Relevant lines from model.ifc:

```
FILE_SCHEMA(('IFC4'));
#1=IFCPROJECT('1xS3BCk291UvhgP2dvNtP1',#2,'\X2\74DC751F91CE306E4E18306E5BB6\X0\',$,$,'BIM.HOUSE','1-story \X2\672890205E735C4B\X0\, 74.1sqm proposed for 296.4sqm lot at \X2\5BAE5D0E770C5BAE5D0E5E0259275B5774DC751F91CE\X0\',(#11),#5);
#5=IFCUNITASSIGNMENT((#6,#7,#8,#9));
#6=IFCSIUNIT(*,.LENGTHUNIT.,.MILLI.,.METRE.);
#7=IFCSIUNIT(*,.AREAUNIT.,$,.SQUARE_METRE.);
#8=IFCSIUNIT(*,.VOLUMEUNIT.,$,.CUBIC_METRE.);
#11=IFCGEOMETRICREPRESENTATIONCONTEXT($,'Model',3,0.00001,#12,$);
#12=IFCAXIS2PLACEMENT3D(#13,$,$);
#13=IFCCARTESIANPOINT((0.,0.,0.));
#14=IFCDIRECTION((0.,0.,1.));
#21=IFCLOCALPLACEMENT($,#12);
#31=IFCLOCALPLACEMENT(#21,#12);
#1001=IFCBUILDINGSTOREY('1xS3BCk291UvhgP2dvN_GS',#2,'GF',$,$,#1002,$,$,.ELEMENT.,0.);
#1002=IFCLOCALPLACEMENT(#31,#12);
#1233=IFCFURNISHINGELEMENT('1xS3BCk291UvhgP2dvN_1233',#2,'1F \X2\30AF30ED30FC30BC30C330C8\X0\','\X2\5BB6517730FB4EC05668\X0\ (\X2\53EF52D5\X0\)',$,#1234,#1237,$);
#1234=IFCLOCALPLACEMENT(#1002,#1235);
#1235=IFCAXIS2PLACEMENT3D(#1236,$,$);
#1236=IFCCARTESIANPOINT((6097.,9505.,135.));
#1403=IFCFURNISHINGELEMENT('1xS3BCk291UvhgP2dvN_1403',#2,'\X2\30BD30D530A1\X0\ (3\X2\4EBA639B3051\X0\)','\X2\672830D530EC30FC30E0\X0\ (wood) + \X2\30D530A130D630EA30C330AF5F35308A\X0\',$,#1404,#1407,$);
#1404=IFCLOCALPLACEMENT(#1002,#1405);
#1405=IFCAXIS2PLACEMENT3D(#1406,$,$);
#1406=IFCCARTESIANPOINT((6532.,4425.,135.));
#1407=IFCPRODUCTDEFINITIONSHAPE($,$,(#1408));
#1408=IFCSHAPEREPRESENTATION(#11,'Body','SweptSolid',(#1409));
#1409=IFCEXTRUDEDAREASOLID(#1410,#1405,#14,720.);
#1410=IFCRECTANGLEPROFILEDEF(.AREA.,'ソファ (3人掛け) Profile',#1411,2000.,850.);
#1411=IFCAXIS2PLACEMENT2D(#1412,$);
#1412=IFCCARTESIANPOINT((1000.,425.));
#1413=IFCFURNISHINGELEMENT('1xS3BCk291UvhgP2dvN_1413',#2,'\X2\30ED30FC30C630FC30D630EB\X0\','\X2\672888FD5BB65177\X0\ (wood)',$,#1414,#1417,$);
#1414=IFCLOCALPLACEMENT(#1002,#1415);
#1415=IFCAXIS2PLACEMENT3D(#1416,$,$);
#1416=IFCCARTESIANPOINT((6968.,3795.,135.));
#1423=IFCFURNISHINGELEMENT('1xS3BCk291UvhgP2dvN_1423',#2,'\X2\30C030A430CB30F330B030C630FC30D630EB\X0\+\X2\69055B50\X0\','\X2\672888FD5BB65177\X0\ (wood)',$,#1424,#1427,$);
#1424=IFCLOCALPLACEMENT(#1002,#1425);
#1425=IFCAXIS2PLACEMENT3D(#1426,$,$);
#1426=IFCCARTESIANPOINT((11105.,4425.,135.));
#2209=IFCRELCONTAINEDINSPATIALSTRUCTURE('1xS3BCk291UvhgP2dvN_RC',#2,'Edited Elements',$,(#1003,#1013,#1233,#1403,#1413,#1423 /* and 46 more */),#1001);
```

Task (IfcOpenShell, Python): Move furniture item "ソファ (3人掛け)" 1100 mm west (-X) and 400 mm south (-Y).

```python
import ifcopenshell
import ifcopenshell.api.geometry
import ifcopenshell.util.placement

model = ifcopenshell.open("model.ifc")

item = model.by_guid("1xS3BCk291UvhgP2dvN_1403")
matrix = ifcopenshell.util.placement.get_local_placement(item.ObjectPlacement)
matrix[0, 3] -= 1100.0
matrix[1, 3] -= 400.0
ifcopenshell.api.geometry.edit_object_placement(model, product=item, matrix=matrix, is_si=False)

print(ifcopenshell.util.placement.get_local_placement(item.ObjectPlacement).round(3) + 0.0)

model.write("model_rev.ifc")
```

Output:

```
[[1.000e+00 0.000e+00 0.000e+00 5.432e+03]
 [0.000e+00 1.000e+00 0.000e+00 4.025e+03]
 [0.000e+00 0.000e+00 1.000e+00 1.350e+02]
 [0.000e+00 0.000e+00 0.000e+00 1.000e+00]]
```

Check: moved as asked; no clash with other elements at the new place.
